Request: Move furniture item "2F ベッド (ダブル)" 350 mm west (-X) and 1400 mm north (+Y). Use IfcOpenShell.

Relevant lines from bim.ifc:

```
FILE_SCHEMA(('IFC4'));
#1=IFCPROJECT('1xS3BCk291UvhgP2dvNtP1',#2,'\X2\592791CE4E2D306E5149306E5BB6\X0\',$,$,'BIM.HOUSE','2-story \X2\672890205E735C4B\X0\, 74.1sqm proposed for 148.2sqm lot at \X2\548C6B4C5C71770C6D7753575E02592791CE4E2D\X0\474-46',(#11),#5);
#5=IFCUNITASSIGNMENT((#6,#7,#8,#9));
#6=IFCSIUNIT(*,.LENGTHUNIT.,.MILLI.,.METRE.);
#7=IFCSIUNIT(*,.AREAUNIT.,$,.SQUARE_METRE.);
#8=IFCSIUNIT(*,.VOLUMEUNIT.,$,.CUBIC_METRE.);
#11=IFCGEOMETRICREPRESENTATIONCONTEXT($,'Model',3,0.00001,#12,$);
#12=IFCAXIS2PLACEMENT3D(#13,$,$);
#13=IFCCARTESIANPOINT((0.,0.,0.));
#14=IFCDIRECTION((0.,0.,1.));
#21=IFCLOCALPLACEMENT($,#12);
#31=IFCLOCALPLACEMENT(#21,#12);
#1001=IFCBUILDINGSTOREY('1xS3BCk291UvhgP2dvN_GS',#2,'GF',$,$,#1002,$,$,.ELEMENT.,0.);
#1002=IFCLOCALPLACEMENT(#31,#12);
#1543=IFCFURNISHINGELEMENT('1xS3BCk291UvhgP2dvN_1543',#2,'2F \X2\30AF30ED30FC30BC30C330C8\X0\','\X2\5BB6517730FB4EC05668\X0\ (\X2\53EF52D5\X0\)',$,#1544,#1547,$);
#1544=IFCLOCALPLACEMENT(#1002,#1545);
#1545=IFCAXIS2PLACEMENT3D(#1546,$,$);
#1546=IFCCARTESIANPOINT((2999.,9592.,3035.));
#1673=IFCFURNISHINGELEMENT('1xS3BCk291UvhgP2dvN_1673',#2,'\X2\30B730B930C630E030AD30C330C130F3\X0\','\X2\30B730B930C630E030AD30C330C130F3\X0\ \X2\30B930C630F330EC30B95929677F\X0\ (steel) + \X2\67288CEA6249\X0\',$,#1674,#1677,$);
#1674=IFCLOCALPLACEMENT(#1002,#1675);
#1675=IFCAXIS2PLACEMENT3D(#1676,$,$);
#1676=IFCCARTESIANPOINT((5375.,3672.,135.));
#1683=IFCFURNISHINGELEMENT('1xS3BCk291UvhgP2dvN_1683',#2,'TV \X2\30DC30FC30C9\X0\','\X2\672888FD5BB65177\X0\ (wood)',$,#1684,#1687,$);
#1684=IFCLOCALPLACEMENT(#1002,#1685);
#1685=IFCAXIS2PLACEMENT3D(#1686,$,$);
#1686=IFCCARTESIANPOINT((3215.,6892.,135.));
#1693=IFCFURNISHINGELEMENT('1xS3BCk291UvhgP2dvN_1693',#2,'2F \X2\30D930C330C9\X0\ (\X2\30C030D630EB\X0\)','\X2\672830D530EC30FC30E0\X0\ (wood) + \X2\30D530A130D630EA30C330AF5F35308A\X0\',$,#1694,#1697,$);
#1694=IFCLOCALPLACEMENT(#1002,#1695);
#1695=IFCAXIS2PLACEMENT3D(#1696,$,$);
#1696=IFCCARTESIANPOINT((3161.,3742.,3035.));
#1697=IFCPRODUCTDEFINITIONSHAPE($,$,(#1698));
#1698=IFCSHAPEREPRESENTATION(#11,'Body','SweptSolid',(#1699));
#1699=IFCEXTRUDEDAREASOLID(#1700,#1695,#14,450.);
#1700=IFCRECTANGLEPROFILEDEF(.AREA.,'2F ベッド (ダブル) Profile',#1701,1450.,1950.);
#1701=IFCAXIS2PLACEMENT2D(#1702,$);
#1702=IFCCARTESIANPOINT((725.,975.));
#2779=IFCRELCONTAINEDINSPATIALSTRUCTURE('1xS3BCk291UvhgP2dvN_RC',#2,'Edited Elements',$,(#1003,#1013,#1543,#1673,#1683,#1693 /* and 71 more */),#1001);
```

```python
import ifcopenshell
import ifcopenshell.api.geometry
import ifcopenshell.util.placement

model = ifcopenshell.open("bim.ifc")

item = model.by_guid("1xS3BCk291UvhgP2dvN_1693")
matrix = ifcopenshell.util.placement.get_local_placement(item.ObjectPlacement)
matrix[0, 3] -= 350.0
matrix[1, 3] += 1400.0
ifcopenshell.api.geometry.edit_object_placement(model, product=item, matrix=matrix, is_si=False)

print(ifcopenshell.util.placement.get_local_placement(item.ObjectPlacement).round(3) + 0.0)

model.write("bim_v2.ifc")
```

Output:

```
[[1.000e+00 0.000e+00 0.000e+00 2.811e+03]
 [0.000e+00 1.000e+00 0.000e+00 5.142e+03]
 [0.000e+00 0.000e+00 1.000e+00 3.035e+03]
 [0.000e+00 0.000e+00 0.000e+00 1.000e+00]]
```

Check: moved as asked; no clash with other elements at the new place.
